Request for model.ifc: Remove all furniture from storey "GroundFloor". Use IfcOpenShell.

First a look at what the model holds.

```python
import ifcopenshell
import ifcopenshell.util.element

model = ifcopenshell.open("model.ifc")
print(model.schema)
storey = next(s for s in model.by_type("IfcBuildingStorey") if s.Name == "GroundFloor")
furniture = [e for e in ifcopenshell.util.element.get_decomposition(storey) if e.is_a("IfcFurnishingElement")]
seen = {}
for e in furniture:
    element_type = ifcopenshell.util.element.get_type(e)
    name = element_type.Name if element_type not in (None, e) else None
    seen[name] = seen.get(name, 0) + 1
for name, count in sorted(seen.items(), key=str):
    print(count, "x", name)
```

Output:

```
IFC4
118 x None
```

```python
import ifcopenshell
import ifcopenshell.api.root
import ifcopenshell.util.element

model = ifcopenshell.open("model.ifc")

storey = next(s for s in model.by_type("IfcBuildingStorey") if s.Name == "GroundFloor")
furniture = [e for e in ifcopenshell.util.element.get_decomposition(storey) if e.is_a("IfcFurnishingElement")]

for e in furniture:
    ifcopenshell.api.root.remove_product(model, product=e)
print(len(furniture), "removed")

model.write("model-out.ifc")
```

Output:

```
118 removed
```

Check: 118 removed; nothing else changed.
